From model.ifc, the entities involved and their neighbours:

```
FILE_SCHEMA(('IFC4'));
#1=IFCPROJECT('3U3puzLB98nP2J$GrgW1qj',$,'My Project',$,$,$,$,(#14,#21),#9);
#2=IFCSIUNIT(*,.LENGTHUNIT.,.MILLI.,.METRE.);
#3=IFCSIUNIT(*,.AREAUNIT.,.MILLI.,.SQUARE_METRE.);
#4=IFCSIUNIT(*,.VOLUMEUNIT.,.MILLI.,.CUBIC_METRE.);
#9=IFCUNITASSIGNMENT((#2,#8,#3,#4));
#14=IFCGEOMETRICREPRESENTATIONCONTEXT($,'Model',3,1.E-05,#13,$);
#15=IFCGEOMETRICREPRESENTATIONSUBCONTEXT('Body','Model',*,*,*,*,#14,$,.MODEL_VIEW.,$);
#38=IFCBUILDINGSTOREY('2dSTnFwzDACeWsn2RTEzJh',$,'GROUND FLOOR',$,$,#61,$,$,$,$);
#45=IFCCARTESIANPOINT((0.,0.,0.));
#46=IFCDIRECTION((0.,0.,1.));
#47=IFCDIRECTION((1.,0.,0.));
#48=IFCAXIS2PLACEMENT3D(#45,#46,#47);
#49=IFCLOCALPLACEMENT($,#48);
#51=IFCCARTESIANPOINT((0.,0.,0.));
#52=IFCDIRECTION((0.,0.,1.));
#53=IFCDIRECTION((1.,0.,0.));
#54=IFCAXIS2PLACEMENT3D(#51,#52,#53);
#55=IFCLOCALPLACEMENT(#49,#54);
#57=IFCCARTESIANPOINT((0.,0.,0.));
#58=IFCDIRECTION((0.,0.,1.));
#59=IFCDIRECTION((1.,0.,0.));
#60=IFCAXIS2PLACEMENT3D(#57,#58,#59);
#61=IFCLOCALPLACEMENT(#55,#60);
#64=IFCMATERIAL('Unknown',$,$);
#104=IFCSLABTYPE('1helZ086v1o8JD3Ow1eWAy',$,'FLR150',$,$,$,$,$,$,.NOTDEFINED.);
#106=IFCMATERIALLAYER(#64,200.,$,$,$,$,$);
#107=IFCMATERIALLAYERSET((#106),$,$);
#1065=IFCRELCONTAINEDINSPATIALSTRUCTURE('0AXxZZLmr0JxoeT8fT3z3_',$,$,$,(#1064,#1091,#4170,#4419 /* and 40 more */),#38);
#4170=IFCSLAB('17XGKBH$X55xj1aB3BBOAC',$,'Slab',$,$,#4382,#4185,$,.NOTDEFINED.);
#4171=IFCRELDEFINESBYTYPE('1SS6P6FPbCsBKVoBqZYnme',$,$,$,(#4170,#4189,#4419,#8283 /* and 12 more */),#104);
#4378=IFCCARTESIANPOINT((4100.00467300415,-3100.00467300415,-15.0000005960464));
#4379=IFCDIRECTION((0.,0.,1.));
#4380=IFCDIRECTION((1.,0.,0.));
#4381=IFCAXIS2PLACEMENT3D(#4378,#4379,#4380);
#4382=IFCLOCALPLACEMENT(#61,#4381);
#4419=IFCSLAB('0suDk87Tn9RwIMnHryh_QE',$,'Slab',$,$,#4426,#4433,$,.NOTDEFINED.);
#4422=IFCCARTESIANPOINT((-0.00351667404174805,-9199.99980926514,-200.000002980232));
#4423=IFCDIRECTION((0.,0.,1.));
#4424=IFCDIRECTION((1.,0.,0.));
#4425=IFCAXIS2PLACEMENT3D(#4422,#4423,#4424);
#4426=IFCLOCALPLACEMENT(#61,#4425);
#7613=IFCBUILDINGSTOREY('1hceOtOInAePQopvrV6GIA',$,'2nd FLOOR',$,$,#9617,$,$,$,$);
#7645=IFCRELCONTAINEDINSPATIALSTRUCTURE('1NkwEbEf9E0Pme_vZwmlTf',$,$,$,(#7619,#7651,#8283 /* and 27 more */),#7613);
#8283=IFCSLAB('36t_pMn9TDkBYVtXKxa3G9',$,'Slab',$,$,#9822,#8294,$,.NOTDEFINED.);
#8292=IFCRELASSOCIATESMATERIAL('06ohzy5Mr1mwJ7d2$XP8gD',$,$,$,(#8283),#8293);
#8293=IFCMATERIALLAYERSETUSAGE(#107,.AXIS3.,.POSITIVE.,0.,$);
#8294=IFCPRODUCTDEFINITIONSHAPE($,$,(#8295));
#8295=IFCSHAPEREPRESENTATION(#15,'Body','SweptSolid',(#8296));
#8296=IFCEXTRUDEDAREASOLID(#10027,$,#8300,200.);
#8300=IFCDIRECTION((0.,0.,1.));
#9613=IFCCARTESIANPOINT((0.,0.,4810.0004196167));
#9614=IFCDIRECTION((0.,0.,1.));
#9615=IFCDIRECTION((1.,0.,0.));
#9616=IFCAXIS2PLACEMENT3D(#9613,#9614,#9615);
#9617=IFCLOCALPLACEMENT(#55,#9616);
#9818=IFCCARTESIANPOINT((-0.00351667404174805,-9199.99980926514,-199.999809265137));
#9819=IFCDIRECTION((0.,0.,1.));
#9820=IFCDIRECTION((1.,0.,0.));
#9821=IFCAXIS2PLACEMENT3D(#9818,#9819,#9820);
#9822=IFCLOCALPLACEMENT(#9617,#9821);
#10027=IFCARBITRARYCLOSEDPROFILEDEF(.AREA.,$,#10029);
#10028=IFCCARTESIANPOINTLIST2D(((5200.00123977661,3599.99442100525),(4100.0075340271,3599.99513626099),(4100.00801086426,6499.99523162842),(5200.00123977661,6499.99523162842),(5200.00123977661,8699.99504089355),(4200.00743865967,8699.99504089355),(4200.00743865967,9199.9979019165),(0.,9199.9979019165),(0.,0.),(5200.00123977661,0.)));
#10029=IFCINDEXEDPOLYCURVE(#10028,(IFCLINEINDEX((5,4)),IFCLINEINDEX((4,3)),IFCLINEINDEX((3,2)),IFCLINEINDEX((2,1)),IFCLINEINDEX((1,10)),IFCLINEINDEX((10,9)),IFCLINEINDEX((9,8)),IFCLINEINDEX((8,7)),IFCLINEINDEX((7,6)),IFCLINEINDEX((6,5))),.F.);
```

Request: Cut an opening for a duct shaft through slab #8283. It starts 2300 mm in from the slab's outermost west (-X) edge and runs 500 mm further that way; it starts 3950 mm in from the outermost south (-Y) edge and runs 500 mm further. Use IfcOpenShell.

```python
import numpy as np
import ifcopenshell
import ifcopenshell.api.feature
import ifcopenshell.api.geometry
import ifcopenshell.api.root
import ifcopenshell.geom
import ifcopenshell.util.placement
import ifcopenshell.util.representation
import ifcopenshell.util.shape
import ifcopenshell.util.unit

model = ifcopenshell.open("model.ifc")
unit_scale = ifcopenshell.util.unit.calculate_unit_scale(model)
settings = ifcopenshell.geom.settings()


def volume(element):
    """Net volume in cubic metres, openings subtracted."""
    shape = ifcopenshell.geom.create_shape(settings, element)
    return ifcopenshell.util.shape.get_volume(shape.geometry)


slab = model.by_guid("36t_pMn9TDkBYVtXKxa3G9")
before = volume(slab)

# Extent in the slab's own axes, in metres. The edges named are its -X and -Y sides.
slab_shape = ifcopenshell.geom.create_shape(settings, slab)
vertices = ifcopenshell.util.shape.get_vertices(slab_shape.geometry)
x_min, y_min, bottom = vertices.min(axis=0)
top = vertices[:, 2].max()

opening = ifcopenshell.api.root.create_entity(model, ifc_class="IfcOpeningElement", name="Duct shaft opening", predefined_type="OPENING")
context = ifcopenshell.util.representation.get_context(model, "Model", "Body", "MODEL_VIEW")
width, depth = 0.5, 0.5
outline = [(0.0, 0.0), (width, 0.0), (width, depth), (0.0, depth), (0.0, 0.0)]
# Overshoot both faces by 50 mm so the cut is clean.
shape = ifcopenshell.api.geometry.add_slab_representation(
    model, context=context, depth=top - bottom + 0.1, polyline=outline
)
ifcopenshell.api.geometry.assign_representation(model, product=opening, representation=shape)

matrix = ifcopenshell.util.placement.get_local_placement(slab.ObjectPlacement)
matrix[:, 3] = matrix @ np.append(np.array([x_min + 2.3, y_min + 3.95, bottom - 0.05]) / unit_scale, 1.0)
ifcopenshell.api.geometry.edit_object_placement(model, product=opening, matrix=matrix, is_si=False)
ifcopenshell.api.feature.add_feature(model, feature=opening, element=slab)

after = volume(slab)

print(f"slab volume {before:.3f} -> {after:.3f} m3")

model.write("model-out.ifc")
```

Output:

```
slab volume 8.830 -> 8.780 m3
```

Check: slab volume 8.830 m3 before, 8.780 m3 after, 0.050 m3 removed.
